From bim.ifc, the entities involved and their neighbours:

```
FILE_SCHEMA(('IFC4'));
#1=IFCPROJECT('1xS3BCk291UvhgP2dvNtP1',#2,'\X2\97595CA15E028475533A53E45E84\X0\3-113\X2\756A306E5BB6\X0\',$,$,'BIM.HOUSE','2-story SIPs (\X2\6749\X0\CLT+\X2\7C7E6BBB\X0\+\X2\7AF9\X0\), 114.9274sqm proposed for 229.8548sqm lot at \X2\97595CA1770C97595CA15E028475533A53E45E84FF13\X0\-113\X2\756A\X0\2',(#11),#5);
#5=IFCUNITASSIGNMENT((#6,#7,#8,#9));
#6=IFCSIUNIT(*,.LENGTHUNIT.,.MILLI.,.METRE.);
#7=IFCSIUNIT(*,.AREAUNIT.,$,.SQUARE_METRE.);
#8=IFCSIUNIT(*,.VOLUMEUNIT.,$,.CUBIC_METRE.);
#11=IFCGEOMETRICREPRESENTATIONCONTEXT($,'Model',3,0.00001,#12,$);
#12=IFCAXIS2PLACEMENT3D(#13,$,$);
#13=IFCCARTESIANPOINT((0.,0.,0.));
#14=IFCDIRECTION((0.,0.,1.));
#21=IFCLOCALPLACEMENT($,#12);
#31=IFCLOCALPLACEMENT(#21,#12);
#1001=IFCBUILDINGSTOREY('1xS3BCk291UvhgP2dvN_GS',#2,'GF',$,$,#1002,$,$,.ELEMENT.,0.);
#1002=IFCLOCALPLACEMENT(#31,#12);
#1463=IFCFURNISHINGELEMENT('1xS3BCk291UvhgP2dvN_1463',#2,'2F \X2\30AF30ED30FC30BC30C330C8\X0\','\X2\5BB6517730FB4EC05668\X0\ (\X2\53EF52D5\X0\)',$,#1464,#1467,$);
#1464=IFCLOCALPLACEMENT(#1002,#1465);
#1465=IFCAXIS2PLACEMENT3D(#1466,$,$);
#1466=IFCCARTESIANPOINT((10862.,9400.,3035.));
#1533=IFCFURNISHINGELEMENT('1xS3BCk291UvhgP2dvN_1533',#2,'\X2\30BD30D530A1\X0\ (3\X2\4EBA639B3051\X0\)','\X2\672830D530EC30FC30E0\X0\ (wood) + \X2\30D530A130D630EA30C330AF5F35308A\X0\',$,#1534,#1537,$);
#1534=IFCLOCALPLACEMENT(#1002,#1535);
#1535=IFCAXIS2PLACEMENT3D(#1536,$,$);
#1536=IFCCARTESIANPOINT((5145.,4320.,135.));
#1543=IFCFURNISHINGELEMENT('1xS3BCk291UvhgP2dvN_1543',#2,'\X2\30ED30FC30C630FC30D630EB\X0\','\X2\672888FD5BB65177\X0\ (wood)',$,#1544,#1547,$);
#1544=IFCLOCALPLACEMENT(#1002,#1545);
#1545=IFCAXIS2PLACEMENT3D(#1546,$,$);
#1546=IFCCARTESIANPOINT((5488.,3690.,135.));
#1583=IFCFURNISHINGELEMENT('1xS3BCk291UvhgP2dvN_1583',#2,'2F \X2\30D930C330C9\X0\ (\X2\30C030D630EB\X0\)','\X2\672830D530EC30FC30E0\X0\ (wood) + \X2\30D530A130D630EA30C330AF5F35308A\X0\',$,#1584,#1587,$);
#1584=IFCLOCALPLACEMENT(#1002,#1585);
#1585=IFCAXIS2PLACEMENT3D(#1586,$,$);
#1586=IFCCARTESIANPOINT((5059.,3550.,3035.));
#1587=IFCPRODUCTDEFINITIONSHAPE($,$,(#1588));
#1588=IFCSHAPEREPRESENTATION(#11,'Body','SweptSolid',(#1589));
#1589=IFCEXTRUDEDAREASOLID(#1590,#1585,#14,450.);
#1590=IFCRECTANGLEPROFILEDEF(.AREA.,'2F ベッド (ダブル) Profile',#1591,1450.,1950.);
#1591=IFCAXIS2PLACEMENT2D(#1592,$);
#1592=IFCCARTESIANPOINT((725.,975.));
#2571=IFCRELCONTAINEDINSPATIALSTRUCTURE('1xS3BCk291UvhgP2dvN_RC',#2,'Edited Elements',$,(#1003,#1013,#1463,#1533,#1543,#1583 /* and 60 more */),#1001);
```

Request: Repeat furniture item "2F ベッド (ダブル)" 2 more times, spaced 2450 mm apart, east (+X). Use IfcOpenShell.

```python
import numpy as np
import ifcopenshell
import ifcopenshell.api.geometry
import ifcopenshell.api.root
import ifcopenshell.util.element
import ifcopenshell.util.placement

model = ifcopenshell.open("bim.ifc")


def reuse_history(source, copy):
    """copy_class also copies each property set's owner history, people and application; keep the originals."""
    for rel in copy.IsDefinedBy:
        if rel.is_a("IfcRelDefinesByProperties") and (history := rel.RelatingPropertyDefinition.OwnerHistory):
            rel.RelatingPropertyDefinition.OwnerHistory = source.OwnerHistory
            ifcopenshell.util.element.remove_deep2(model, history)


source = model.by_id(1583)
base = ifcopenshell.util.placement.get_local_placement(source.ObjectPlacement)
step = np.array([1.0, 0.0, 0.0]) * 2450.0

for i in range(1, 3):
    copy = ifcopenshell.api.root.copy_class(model, product=source)
    copy.Representation = ifcopenshell.util.element.copy_deep(
        model, source.Representation, exclude=["IfcGeometricRepresentationContext", "IfcRepresentationMap"]
    )
    reuse_history(source, copy)
    matrix = base.copy()
    matrix[:3, 3] += i * step
    print("added at", matrix[:3, 3].round(3) + 0.0)
    ifcopenshell.api.geometry.edit_object_placement(model, product=copy, matrix=matrix, is_si=False)

model.write("bim-out.ifc")
```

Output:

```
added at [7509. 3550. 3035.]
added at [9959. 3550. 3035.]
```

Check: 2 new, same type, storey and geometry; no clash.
